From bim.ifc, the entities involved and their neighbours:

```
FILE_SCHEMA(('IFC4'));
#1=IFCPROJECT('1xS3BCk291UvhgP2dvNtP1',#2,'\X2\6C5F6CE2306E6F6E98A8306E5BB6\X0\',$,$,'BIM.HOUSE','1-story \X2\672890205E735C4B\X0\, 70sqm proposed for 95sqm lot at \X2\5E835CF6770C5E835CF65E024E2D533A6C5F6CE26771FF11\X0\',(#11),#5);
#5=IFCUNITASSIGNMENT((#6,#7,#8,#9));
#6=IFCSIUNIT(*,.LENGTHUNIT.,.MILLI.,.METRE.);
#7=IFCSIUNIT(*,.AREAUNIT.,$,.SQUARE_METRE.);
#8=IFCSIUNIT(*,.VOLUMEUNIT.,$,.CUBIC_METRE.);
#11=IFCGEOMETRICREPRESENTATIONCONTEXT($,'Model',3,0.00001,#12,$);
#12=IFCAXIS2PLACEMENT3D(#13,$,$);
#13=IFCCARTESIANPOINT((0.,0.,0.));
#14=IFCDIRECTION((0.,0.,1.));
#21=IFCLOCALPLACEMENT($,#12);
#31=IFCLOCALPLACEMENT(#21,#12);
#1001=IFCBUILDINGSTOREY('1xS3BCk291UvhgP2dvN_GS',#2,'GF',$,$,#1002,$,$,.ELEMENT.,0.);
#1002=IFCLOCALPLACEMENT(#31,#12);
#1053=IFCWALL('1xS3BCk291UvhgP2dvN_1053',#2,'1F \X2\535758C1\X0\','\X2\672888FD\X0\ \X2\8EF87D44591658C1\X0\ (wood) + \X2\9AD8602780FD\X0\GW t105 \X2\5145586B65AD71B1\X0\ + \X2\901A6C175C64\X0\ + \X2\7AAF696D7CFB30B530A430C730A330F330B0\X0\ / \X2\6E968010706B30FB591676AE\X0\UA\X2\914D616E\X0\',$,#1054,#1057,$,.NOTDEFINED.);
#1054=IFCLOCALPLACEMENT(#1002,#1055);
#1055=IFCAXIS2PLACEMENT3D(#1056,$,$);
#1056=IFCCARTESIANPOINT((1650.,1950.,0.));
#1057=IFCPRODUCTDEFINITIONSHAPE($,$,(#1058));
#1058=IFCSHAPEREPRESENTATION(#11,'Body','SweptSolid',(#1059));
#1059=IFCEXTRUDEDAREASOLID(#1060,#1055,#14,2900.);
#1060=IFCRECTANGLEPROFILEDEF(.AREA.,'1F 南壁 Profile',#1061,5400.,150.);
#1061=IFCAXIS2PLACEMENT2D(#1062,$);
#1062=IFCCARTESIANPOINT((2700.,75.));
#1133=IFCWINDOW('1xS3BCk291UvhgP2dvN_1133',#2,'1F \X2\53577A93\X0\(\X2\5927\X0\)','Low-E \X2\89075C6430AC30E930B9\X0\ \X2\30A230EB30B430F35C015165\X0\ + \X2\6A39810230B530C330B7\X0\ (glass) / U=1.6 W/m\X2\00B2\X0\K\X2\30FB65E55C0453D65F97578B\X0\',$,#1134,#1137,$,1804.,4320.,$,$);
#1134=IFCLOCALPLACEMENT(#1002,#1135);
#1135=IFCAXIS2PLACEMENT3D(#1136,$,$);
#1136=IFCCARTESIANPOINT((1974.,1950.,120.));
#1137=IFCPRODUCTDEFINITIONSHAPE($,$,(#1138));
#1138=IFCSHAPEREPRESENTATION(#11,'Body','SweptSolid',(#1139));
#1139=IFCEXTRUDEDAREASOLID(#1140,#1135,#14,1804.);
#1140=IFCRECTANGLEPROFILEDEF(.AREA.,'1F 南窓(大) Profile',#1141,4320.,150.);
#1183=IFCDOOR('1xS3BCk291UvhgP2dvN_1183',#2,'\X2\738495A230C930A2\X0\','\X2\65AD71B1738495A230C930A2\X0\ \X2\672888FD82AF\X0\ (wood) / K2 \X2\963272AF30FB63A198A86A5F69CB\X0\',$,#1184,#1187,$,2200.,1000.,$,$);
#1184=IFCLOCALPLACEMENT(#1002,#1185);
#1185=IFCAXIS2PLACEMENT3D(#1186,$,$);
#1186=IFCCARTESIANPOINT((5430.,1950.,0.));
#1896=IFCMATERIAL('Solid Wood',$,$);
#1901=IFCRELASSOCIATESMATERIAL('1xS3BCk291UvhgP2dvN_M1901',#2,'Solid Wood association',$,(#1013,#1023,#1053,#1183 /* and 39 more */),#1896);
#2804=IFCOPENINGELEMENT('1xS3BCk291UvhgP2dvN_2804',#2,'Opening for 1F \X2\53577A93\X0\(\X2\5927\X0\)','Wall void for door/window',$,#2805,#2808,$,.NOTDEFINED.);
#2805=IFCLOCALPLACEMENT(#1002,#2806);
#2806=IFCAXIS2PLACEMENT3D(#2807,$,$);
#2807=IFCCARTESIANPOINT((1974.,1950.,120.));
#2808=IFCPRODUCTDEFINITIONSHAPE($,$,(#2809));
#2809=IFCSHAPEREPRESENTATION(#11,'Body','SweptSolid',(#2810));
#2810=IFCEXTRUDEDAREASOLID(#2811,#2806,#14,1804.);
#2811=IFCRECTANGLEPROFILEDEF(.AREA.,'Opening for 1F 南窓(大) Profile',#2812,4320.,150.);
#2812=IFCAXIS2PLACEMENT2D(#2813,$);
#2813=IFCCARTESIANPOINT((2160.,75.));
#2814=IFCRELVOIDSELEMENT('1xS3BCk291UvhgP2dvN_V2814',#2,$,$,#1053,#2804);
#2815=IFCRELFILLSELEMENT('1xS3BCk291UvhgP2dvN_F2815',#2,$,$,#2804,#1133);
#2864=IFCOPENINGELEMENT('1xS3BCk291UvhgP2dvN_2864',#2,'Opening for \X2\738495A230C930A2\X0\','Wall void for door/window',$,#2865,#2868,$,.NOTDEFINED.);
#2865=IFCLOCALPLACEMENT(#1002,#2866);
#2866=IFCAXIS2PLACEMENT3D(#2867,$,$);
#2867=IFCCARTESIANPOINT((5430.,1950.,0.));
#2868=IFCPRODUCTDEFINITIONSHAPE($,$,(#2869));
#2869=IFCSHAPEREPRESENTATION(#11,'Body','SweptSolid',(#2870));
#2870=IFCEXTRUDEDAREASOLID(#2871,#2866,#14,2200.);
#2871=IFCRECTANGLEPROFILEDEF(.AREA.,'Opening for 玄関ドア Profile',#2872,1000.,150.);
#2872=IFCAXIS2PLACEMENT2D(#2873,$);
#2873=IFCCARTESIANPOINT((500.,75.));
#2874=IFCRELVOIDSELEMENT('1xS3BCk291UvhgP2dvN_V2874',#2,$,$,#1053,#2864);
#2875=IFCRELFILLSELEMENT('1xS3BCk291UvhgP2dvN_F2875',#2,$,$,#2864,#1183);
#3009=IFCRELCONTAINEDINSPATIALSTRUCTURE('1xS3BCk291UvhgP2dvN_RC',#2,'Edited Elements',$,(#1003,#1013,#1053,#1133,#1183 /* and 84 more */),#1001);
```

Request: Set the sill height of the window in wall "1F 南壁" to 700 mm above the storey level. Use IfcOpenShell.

```python
import numpy as np
import ifcopenshell
import ifcopenshell.api.geometry
import ifcopenshell.geom
import ifcopenshell.util.element
import ifcopenshell.util.placement
import ifcopenshell.util.shape
import ifcopenshell.util.unit

model = ifcopenshell.open("bim.ifc")
unit_scale = ifcopenshell.util.unit.calculate_unit_scale(model)

window = model.by_guid("1xS3BCk291UvhgP2dvN_1133")
opening = window.FillsVoids[0].RelatingOpeningElement
storey = ifcopenshell.util.element.get_container(window, ifc_class="IfcBuildingStorey")
level = ifcopenshell.util.placement.get_local_placement(storey.ObjectPlacement)[2, 3]

# The opening's origin need not be at the sill, so measure its lowest point.
shape = ifcopenshell.geom.create_shape(ifcopenshell.geom.settings(), opening)
bottom = ifcopenshell.util.shape.get_shape_bottom_elevation(shape, shape.geometry) / unit_scale
dz = level + 0.7 / unit_scale - bottom

shift = np.array([0.0, 0.0, dz])
# The window is not placed relative to its opening, so move both.
for product in (opening, window):
    matrix = ifcopenshell.util.placement.get_local_placement(product.ObjectPlacement)
    matrix[:3, 3] += shift
    ifcopenshell.api.geometry.edit_object_placement(model, product=product, matrix=matrix, is_si=False)

print(f"moved by {dz * unit_scale:+.3f} m")

model.write("bim_rev.ifc")
```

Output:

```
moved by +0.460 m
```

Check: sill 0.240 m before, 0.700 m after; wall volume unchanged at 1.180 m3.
